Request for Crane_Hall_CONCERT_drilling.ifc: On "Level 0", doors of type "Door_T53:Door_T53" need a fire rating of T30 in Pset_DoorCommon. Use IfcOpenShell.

First a look at what the model holds.

```python
import ifcopenshell
import ifcopenshell.util.element

model = ifcopenshell.open("Crane_Hall_CONCERT_drilling.ifc")
print(model.schema)
storey = next(s for s in model.by_type("IfcBuildingStorey") if s.Name == "Level 0")
doors = [e for e in ifcopenshell.util.element.get_decomposition(storey) if e.is_a("IfcDoor")]
seen = {}
for e in doors:
    element_type = ifcopenshell.util.element.get_type(e)
    key = (element_type.Name if element_type != e and element_type else None, ifcopenshell.util.element.get_pset(e, "Pset_DoorCommon", "FireRating"))
    seen[key] = seen.get(key, 0) + 1
for (name, value), count in sorted(seen.items(), key=str):
    print(count, "x", name, "|", value)
```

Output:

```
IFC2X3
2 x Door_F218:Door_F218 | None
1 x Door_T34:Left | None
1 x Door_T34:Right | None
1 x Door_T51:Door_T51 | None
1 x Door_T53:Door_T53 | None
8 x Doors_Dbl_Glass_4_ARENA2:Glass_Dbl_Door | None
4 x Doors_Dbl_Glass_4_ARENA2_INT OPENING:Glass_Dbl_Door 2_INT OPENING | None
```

```python
import ifcopenshell
import ifcopenshell.api.pset
import ifcopenshell.util.element

model = ifcopenshell.open("Crane_Hall_CONCERT_drilling.ifc")

storey = next(s for s in model.by_type("IfcBuildingStorey") if s.Name == "Level 0")
doors = [e for e in ifcopenshell.util.element.get_decomposition(storey) if e.is_a("IfcDoor")]

count = 0
for e in doors:
    element_type = ifcopenshell.util.element.get_type(e)
    if element_type in (None, e) or element_type.Name != "Door_T53:Door_T53":
        continue
    # add_pset returns the element's existing set when there is one.
    pset = ifcopenshell.api.pset.add_pset(model, product=e, name="Pset_DoorCommon")
    ifcopenshell.api.pset.edit_pset(model, pset=pset, properties={"FireRating": "T30"})
    count += 1

print(count, "doors updated")

model.write("Crane_Hall_CONCERT_drilling_rev.ifc")
```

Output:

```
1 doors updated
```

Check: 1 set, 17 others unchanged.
